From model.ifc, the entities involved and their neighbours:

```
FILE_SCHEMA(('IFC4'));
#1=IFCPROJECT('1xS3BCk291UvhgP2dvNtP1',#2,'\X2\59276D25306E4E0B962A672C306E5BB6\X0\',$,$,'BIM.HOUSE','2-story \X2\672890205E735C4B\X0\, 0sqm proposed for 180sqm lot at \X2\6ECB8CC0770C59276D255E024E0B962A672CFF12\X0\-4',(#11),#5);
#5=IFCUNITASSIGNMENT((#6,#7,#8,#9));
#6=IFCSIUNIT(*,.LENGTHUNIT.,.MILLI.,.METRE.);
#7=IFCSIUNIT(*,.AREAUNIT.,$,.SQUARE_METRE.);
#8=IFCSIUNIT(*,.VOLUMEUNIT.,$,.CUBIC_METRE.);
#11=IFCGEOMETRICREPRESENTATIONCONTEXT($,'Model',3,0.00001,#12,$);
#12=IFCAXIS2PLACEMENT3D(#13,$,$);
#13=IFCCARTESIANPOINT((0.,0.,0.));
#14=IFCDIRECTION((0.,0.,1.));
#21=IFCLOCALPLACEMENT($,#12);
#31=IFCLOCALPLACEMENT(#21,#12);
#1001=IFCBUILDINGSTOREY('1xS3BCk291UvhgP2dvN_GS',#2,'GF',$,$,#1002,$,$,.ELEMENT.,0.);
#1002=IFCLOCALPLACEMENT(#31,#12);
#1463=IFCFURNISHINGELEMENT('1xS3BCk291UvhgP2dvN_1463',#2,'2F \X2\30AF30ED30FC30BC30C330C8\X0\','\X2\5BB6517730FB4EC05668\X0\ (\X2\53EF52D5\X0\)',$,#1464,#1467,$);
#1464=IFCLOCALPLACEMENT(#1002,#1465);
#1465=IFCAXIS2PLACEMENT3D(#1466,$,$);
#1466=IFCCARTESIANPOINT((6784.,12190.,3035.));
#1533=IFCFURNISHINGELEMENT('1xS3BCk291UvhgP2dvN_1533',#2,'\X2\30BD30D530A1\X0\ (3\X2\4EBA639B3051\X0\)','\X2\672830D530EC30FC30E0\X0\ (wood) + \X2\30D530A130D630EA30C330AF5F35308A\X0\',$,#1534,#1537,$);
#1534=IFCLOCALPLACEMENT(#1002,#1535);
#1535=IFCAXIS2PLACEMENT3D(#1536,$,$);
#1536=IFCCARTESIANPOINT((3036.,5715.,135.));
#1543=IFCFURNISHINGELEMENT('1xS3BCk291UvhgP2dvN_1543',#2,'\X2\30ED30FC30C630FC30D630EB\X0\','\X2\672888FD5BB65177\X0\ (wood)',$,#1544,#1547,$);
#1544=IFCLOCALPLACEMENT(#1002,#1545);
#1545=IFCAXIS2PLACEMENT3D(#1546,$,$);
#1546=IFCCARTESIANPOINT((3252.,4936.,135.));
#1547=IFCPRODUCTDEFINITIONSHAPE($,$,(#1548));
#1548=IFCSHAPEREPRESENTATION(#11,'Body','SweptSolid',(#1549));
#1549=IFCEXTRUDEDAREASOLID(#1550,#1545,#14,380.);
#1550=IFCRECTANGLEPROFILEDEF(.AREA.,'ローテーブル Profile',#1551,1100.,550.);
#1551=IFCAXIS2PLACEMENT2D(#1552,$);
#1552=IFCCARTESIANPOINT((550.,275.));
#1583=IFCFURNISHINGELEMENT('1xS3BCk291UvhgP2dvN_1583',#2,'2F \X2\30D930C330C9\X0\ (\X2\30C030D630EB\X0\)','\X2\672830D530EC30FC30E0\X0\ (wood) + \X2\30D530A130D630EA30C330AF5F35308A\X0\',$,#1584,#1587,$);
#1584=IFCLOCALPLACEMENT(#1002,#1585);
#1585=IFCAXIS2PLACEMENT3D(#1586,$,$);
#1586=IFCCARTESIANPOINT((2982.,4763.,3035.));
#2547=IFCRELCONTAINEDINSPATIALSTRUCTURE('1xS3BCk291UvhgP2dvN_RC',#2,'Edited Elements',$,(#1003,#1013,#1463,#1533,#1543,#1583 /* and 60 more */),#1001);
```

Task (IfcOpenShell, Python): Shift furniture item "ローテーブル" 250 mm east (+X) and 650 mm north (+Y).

```python
import ifcopenshell
import ifcopenshell.api.geometry
import ifcopenshell.util.placement
import ifcopenshell.util.unit

model = ifcopenshell.open("model.ifc")
unit_scale = ifcopenshell.util.unit.calculate_unit_scale(model)

item = model.by_guid("1xS3BCk291UvhgP2dvN_1543")
matrix = ifcopenshell.util.placement.get_local_placement(item.ObjectPlacement)
matrix[0, 3] += 0.25 / unit_scale
matrix[1, 3] += 0.65 / unit_scale
ifcopenshell.api.geometry.edit_object_placement(model, product=item, matrix=matrix, is_si=False)

print(ifcopenshell.util.placement.get_local_placement(item.ObjectPlacement).round(3) + 0.0)

model.write("model_updated.ifc")
```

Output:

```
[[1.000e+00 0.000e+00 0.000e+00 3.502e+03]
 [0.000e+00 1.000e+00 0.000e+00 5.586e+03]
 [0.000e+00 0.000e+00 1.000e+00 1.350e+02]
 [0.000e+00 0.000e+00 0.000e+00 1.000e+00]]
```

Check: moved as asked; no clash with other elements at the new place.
